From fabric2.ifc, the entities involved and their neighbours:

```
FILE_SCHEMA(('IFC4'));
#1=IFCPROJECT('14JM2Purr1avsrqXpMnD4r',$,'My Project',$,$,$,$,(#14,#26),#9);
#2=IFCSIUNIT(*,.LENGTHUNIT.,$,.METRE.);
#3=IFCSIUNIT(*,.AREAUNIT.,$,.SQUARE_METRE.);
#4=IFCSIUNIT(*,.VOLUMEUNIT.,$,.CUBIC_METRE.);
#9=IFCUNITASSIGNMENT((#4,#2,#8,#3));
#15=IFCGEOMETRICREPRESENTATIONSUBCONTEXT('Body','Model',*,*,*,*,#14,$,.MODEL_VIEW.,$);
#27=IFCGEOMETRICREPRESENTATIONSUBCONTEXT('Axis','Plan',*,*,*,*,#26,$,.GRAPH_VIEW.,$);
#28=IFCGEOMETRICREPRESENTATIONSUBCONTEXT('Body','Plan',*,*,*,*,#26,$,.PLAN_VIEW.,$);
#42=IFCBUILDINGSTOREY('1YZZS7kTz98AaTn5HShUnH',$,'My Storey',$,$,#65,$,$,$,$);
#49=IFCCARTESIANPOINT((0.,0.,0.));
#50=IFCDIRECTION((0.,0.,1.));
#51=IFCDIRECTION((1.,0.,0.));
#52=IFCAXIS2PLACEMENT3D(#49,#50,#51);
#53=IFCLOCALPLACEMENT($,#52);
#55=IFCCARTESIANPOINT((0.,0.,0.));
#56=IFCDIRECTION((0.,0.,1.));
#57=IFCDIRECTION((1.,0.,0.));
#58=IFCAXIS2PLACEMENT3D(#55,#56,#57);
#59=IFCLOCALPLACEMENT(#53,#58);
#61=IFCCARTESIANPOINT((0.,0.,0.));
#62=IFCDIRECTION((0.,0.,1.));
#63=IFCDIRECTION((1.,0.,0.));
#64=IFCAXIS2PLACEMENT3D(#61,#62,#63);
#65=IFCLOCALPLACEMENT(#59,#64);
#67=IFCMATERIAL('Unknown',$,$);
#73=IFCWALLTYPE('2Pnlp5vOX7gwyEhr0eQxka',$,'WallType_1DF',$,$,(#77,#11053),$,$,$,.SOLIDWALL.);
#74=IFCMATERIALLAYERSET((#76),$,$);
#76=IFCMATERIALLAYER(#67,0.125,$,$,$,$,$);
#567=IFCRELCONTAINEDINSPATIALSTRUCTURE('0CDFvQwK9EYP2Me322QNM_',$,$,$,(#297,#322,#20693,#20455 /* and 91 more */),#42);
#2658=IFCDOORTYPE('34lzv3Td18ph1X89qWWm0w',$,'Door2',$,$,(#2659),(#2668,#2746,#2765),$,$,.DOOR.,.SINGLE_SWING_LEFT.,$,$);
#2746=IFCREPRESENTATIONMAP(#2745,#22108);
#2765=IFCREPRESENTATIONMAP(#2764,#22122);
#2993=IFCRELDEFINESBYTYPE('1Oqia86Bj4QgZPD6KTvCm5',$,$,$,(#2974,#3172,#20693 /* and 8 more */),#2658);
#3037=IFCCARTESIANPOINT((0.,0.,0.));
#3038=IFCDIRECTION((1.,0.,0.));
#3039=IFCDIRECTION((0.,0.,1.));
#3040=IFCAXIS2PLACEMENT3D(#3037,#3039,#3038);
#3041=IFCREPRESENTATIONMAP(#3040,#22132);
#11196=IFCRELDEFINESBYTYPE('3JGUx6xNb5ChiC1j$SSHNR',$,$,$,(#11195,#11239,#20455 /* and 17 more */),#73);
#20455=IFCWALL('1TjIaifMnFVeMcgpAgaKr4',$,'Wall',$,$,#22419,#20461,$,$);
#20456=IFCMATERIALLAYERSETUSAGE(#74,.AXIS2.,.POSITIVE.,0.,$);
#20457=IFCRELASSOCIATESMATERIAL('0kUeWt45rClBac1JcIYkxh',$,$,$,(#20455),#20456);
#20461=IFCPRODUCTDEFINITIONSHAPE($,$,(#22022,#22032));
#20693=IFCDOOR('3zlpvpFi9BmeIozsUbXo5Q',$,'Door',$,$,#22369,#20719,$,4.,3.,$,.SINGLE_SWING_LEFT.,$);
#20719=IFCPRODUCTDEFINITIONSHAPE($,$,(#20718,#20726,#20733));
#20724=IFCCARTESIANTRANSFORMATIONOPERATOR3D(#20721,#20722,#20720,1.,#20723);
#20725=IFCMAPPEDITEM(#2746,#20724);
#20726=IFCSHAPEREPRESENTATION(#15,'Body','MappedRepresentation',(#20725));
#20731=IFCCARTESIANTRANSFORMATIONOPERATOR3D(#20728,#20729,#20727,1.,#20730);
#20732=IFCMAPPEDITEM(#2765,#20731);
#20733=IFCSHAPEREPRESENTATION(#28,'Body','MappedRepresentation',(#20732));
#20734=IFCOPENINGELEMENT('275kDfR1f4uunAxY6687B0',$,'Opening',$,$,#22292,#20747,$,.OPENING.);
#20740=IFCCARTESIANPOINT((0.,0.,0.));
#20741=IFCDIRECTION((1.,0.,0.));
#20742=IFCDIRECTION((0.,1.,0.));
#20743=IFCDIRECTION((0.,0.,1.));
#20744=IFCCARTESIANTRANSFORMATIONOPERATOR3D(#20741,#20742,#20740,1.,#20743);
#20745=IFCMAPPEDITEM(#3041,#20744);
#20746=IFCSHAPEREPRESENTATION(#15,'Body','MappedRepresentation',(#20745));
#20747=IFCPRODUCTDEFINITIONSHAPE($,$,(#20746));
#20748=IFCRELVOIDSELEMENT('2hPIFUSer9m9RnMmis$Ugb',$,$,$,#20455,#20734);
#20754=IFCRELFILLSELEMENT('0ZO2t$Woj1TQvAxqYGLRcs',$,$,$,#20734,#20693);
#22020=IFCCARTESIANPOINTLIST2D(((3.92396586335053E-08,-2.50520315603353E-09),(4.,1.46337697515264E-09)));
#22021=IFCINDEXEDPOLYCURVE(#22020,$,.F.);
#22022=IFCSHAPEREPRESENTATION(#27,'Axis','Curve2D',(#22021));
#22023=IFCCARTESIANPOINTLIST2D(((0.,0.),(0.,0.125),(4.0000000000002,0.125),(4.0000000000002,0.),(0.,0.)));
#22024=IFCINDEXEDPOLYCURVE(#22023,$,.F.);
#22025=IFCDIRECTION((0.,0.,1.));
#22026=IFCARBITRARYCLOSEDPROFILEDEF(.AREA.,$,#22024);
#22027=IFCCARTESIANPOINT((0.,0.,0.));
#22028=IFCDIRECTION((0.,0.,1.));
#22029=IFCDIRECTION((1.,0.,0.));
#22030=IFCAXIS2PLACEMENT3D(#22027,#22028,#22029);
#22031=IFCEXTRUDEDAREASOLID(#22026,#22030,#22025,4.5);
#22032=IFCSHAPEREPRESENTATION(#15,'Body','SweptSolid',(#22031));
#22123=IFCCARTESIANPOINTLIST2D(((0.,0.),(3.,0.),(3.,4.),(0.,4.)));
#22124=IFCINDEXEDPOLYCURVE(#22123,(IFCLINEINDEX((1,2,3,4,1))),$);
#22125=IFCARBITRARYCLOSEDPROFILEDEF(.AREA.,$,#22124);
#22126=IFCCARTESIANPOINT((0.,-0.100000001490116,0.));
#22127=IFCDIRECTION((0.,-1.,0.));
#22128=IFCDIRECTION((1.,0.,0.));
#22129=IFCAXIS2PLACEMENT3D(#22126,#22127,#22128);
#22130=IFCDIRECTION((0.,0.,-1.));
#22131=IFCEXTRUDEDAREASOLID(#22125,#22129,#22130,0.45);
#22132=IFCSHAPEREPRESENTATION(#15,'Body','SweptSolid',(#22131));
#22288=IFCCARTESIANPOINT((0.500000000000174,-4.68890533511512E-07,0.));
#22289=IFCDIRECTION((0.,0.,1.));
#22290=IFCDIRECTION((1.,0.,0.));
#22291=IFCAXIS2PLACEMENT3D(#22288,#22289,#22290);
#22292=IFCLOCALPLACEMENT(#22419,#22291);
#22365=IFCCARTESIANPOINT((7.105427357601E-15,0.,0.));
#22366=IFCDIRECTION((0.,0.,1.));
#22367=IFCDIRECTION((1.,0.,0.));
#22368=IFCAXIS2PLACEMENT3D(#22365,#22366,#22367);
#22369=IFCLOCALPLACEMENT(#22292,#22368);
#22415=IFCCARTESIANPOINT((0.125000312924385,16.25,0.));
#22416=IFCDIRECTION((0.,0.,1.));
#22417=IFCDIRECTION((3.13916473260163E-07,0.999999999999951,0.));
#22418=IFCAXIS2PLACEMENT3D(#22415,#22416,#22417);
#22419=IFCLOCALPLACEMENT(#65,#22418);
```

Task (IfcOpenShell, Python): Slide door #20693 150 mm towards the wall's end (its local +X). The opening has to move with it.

```python
import ifcopenshell
import ifcopenshell.api.geometry
import ifcopenshell.util.placement

model = ifcopenshell.open("fabric2.ifc")

door = model.by_id(20693)
opening = door.FillsVoids[0].RelatingOpeningElement
wall = opening.VoidsElements[0].RelatingBuildingElement

wall_matrix = ifcopenshell.util.placement.get_local_placement(wall.ObjectPlacement)
shift = wall_matrix[:3, 0] * 0.15
before = ifcopenshell.util.placement.get_local_placement(door.ObjectPlacement)[:3, 3].copy()

# The door is placed relative to its opening, so it follows when the opening moves.
matrix = ifcopenshell.util.placement.get_local_placement(opening.ObjectPlacement)
matrix[:3, 3] += shift
ifcopenshell.api.geometry.edit_object_placement(
    model, product=opening, matrix=matrix, is_si=False, should_transform_children=True
)

after = ifcopenshell.util.placement.get_local_placement(door.ObjectPlacement)[:3, 3]
print("door moved by", (after - before).round(3) + 0.0)

model.write("fabric2_rev.ifc")
```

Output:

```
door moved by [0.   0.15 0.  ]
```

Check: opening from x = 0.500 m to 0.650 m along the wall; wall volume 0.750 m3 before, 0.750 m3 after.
